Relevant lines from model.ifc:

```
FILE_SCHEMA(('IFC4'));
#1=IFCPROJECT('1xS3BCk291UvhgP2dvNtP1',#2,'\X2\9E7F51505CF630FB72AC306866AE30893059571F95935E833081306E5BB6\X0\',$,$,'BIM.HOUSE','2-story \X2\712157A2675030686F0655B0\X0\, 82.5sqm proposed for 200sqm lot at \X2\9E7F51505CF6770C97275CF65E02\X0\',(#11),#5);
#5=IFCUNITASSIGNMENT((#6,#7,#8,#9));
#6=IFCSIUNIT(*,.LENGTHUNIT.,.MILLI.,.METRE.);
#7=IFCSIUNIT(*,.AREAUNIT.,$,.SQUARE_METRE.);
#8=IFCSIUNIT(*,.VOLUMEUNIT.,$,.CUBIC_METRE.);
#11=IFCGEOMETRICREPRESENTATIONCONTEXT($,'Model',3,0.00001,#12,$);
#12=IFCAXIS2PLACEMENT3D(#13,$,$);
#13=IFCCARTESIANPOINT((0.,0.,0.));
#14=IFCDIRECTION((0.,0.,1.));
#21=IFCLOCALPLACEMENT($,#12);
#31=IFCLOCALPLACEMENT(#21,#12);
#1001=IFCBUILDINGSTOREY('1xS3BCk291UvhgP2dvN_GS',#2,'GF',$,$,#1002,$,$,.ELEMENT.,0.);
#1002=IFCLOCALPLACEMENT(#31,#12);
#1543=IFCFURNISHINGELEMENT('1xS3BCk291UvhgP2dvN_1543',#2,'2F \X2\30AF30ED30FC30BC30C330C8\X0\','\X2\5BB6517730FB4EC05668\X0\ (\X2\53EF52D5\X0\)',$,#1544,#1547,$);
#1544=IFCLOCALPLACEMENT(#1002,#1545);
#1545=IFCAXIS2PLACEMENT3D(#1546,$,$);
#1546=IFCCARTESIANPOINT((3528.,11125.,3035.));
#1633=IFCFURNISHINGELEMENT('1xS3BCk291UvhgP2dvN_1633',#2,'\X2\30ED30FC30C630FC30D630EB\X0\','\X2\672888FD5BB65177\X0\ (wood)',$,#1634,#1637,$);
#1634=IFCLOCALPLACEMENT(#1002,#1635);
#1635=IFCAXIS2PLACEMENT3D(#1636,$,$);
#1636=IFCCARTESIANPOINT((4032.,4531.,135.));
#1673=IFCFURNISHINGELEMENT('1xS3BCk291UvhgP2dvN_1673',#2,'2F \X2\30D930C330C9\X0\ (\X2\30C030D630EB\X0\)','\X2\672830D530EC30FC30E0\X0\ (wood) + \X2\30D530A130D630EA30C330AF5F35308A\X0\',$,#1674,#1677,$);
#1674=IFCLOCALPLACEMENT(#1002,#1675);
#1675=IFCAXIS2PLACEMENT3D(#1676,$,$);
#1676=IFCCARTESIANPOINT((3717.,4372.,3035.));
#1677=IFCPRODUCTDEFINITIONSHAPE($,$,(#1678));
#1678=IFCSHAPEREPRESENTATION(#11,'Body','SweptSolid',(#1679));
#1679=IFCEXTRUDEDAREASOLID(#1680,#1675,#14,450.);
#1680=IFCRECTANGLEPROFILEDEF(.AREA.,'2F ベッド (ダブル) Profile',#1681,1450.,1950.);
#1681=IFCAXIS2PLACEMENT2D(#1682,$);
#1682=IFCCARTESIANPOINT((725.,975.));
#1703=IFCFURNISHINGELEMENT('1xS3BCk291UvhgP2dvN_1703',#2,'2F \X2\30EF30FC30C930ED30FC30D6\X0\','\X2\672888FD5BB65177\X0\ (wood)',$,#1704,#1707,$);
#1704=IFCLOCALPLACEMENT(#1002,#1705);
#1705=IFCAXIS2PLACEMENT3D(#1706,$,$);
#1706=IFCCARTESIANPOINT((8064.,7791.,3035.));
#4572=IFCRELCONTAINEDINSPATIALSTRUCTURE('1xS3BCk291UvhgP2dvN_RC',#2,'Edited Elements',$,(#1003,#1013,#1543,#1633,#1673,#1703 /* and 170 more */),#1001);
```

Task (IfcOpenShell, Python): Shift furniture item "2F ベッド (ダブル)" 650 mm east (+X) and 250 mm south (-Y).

```python
import ifcopenshell
import ifcopenshell.api.geometry
import ifcopenshell.util.placement
import ifcopenshell.util.unit

model = ifcopenshell.open("model.ifc")
unit_scale = ifcopenshell.util.unit.calculate_unit_scale(model)

item = model.by_guid("1xS3BCk291UvhgP2dvN_1673")
matrix = ifcopenshell.util.placement.get_local_placement(item.ObjectPlacement)
matrix[0, 3] += 0.65 / unit_scale
matrix[1, 3] -= 0.25 / unit_scale
ifcopenshell.api.geometry.edit_object_placement(model, product=item, matrix=matrix, is_si=False)

print(ifcopenshell.util.placement.get_local_placement(item.ObjectPlacement).round(3) + 0.0)

model.write("model_edited.ifc")
```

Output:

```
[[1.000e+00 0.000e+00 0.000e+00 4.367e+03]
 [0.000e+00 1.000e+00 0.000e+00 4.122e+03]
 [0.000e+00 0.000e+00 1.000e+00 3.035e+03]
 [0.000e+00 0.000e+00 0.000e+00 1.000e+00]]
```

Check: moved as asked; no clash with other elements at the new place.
